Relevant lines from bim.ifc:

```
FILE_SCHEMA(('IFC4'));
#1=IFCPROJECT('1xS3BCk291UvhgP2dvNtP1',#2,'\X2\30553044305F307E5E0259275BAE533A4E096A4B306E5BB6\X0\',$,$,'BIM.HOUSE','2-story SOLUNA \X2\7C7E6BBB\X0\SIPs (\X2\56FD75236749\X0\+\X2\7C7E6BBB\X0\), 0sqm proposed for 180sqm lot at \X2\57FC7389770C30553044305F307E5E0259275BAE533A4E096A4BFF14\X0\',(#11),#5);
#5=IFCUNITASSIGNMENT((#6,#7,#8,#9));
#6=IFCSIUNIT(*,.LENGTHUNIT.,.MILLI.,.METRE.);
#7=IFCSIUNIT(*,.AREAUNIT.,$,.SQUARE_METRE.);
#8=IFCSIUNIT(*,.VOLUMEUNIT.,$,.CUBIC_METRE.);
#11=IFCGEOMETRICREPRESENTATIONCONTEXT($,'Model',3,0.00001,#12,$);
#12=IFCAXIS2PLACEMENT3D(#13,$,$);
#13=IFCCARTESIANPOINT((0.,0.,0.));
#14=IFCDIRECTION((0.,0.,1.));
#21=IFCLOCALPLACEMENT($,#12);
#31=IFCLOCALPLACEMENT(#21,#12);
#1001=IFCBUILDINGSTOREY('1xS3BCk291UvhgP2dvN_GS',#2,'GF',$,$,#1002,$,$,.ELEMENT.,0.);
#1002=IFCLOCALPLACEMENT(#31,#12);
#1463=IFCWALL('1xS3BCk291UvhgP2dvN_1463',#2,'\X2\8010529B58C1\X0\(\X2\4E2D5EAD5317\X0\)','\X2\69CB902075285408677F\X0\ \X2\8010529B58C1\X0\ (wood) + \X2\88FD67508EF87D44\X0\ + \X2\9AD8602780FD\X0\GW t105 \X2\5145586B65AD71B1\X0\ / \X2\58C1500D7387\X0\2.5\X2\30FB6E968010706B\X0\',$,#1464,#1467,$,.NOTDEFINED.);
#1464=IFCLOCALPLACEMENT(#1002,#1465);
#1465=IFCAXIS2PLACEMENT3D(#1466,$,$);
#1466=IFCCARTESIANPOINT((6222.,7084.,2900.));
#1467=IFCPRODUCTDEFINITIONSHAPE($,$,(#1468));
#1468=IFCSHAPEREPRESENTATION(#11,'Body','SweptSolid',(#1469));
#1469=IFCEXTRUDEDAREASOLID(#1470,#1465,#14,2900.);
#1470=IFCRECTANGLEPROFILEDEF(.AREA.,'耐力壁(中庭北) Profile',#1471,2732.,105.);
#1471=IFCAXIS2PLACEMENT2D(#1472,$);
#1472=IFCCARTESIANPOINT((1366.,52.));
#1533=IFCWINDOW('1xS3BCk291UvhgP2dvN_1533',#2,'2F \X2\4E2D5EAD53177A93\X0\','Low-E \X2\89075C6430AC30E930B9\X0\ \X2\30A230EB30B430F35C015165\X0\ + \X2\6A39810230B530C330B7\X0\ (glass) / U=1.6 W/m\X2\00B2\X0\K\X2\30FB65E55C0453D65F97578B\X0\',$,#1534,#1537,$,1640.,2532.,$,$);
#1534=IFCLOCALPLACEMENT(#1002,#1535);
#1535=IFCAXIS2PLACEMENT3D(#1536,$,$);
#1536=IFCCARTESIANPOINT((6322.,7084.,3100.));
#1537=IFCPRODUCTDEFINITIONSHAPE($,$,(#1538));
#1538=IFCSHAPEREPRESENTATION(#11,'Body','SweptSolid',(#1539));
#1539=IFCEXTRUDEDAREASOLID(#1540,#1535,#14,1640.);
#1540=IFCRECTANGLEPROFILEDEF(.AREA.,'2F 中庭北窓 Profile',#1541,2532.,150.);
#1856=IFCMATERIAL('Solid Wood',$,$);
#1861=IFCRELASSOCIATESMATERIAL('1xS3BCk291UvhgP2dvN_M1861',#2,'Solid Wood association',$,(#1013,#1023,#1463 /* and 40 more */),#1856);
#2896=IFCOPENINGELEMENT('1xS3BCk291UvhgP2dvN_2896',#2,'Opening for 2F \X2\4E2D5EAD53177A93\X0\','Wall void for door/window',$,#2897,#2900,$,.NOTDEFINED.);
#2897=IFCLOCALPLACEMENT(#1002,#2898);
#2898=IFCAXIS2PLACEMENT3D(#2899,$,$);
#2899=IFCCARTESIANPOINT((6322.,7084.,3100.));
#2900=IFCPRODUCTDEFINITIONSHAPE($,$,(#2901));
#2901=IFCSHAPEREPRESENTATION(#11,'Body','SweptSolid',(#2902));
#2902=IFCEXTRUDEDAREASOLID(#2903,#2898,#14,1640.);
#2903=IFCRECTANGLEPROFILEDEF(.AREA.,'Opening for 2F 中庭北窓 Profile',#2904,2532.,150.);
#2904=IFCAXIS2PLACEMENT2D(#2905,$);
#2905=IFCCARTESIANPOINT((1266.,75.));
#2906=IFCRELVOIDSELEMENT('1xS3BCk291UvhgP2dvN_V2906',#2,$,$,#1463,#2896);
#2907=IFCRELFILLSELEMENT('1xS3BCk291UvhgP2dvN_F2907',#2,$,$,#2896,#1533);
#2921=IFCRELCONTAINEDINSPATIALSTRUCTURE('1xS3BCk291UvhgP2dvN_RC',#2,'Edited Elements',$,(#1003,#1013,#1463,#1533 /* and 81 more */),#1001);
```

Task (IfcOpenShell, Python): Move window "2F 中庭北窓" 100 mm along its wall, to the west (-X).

```python
import ifcopenshell
import ifcopenshell.api.geometry
import ifcopenshell.util.placement

model = ifcopenshell.open("bim.ifc")

window = model.by_guid("1xS3BCk291UvhgP2dvN_1533")
opening = window.FillsVoids[0].RelatingOpeningElement
wall = opening.VoidsElements[0].RelatingBuildingElement

wall_matrix = ifcopenshell.util.placement.get_local_placement(wall.ObjectPlacement)
shift = wall_matrix[:3, 0] * -100.0
before = ifcopenshell.util.placement.get_local_placement(window.ObjectPlacement)[:3, 3].copy()

# The window is not placed relative to its opening, so move both.
for product in (opening, window):
    matrix = ifcopenshell.util.placement.get_local_placement(product.ObjectPlacement)
    matrix[:3, 3] += shift
    ifcopenshell.api.geometry.edit_object_placement(model, product=product, matrix=matrix, is_si=False)

after = ifcopenshell.util.placement.get_local_placement(window.ObjectPlacement)[:3, 3]
print("window moved by", (after - before).round(3) + 0.0)

model.write("bim_rev.ifc")
```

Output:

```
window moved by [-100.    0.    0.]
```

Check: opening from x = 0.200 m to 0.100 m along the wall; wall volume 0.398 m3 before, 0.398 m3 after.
